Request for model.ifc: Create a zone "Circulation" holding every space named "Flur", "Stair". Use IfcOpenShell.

First a look at what the model holds.

```python
import ifcopenshell

model = ifcopenshell.open("model.ifc")
print(model.schema)
seen = {}
for space in model.by_type("IfcSpace"):
    seen[space.LongName] = seen.get(space.LongName, 0) + 1
for name, count in sorted(seen.items(), key=str):
    print(count, "x", name)
print("zones:", [z.Name for z in model.by_type("IfcZone")][:20])
```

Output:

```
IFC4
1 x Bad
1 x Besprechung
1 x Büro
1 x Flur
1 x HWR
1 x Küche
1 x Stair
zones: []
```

```python
import ifcopenshell
import ifcopenshell.api.group
import ifcopenshell.api.root

model = ifcopenshell.open("model.ifc")

names = {"Flur", "Stair"}
spaces = [s for s in model.by_type("IfcSpace") if s.LongName in names]

zone = ifcopenshell.api.root.create_entity(model, ifc_class="IfcZone", name="Circulation")
ifcopenshell.api.group.assign_group(model, products=spaces, group=zone)
print(len(spaces), "spaces in", zone.Name)

model.write("model_rev.ifc")
```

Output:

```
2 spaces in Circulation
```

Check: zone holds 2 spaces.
